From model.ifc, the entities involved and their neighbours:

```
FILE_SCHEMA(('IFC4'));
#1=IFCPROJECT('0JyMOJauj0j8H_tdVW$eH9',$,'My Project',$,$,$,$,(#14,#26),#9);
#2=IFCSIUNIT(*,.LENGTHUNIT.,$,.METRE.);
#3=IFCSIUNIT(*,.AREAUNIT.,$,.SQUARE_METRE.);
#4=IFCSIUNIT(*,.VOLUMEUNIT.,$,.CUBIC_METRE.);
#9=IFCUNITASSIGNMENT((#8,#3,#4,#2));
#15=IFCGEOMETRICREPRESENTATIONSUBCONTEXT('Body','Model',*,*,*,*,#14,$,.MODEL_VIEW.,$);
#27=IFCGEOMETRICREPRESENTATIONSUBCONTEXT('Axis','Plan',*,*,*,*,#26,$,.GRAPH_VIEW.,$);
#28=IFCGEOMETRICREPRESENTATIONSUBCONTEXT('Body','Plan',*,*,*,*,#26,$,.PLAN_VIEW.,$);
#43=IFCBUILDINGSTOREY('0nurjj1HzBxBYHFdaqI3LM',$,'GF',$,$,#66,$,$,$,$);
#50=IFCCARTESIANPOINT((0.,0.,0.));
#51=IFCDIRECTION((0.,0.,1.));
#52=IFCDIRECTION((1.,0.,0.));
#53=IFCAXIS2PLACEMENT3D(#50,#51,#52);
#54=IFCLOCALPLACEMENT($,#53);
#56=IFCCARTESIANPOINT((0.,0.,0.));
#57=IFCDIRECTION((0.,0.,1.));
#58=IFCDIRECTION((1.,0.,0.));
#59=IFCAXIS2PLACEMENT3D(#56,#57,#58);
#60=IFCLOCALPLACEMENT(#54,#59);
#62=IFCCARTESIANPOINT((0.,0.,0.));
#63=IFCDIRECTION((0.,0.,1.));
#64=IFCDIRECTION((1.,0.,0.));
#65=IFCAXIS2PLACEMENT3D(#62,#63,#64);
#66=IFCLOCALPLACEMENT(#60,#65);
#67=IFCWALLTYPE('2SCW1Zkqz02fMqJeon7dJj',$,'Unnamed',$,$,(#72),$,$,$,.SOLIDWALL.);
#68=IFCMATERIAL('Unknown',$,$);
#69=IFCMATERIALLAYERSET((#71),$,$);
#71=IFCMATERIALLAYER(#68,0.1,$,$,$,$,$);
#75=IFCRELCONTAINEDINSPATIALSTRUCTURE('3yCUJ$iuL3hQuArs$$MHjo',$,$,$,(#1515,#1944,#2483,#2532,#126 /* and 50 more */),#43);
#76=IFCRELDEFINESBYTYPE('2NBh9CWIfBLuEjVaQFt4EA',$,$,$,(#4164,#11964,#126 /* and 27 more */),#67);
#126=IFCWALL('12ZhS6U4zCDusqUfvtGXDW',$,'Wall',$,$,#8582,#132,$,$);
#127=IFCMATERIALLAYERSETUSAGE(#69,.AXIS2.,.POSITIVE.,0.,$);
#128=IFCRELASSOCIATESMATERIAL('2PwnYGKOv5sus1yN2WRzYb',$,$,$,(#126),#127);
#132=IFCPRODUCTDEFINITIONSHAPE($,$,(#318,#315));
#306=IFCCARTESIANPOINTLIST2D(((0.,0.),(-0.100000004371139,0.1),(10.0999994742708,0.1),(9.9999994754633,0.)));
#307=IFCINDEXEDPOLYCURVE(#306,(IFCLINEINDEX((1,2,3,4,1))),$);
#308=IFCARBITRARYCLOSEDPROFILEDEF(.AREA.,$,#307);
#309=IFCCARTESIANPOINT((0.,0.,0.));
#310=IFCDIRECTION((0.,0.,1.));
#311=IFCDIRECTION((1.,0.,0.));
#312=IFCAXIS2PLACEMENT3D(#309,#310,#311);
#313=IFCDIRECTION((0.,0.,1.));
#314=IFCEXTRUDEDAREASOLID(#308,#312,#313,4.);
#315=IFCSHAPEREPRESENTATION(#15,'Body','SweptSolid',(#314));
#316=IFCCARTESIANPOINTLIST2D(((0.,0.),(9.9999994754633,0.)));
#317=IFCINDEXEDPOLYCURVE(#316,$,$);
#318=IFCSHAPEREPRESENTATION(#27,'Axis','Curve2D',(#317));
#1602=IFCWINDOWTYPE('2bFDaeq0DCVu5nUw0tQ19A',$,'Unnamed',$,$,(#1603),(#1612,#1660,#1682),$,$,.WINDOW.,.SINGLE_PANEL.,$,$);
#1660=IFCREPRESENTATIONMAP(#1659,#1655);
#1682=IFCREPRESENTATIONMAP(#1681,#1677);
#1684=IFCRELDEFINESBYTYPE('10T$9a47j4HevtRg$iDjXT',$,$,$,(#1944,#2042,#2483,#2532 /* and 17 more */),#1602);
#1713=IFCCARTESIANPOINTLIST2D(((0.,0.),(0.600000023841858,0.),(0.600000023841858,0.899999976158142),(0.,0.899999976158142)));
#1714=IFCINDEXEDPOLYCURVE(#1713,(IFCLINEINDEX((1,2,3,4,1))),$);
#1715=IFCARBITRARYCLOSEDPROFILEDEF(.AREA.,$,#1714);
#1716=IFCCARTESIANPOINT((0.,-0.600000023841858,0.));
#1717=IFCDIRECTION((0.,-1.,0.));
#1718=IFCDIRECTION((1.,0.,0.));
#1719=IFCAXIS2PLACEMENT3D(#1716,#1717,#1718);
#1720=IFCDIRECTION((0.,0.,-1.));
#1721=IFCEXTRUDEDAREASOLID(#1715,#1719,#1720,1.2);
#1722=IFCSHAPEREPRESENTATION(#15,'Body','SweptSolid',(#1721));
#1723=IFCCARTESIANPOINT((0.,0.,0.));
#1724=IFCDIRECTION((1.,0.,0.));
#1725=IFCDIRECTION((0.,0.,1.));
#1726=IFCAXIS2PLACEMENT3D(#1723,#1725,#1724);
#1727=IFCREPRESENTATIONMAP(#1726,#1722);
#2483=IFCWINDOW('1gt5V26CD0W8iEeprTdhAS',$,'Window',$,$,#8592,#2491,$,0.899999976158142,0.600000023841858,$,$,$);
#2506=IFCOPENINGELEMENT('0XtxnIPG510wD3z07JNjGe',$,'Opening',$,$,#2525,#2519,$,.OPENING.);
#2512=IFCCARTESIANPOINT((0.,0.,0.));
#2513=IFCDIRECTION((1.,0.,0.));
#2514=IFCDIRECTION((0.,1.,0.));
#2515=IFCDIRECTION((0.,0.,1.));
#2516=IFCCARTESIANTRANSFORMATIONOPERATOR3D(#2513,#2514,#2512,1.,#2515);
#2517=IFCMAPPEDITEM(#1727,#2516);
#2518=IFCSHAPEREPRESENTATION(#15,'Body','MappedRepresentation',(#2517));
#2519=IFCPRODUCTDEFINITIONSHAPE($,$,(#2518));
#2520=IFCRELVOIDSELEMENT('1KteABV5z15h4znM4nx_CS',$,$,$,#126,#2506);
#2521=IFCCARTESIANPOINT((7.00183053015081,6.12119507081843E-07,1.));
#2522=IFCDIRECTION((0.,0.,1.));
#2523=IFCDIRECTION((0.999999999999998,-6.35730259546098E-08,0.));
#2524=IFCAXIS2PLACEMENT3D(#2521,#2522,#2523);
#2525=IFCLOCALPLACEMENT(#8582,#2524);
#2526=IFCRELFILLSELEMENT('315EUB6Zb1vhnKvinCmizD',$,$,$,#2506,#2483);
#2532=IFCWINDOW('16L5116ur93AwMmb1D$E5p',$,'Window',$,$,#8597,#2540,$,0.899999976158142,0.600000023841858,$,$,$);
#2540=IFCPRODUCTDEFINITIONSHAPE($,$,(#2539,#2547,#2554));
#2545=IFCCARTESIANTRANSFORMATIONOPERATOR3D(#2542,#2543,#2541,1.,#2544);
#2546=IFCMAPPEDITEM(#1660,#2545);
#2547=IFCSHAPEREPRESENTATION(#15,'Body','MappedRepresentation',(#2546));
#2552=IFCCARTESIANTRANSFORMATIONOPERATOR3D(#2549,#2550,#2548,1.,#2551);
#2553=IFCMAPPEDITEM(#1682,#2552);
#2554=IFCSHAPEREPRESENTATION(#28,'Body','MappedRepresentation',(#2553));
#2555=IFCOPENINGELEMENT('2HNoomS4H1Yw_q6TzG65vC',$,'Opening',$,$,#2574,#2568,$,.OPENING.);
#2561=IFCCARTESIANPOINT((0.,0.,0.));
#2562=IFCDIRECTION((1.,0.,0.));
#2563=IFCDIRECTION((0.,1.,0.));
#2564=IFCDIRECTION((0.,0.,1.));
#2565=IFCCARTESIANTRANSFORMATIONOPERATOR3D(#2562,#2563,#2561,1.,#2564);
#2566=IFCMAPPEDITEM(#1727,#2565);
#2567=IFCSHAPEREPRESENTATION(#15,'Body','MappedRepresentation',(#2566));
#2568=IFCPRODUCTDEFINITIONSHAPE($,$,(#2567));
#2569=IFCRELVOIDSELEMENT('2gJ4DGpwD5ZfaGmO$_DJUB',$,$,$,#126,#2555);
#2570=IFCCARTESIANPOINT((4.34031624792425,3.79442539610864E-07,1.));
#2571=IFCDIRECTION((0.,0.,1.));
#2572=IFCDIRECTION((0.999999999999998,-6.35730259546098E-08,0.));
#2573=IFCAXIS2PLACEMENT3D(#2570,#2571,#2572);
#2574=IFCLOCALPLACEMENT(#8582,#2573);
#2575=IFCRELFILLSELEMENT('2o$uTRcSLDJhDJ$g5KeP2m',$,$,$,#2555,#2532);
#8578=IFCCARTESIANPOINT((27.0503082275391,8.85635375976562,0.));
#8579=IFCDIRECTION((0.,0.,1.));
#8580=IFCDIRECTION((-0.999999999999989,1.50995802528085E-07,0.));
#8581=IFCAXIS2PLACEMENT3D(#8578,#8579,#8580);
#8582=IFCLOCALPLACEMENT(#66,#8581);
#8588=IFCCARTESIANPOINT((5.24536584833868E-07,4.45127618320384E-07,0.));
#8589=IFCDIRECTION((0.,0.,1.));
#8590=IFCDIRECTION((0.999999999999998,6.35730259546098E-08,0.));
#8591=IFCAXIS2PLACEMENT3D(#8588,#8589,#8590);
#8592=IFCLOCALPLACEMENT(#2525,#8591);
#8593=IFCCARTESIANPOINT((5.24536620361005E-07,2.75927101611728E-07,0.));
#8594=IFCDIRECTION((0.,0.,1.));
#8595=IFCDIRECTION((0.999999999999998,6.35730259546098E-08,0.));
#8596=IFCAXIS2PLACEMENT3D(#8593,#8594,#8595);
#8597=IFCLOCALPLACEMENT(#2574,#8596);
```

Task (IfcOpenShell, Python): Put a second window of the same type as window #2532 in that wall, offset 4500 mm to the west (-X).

```python
import ifcopenshell
import ifcopenshell.api.feature
import ifcopenshell.api.geometry
import ifcopenshell.api.root
import ifcopenshell.geom
import ifcopenshell.util.element
import ifcopenshell.util.placement
import ifcopenshell.util.shape
import ifcopenshell.util.unit

model = ifcopenshell.open("model.ifc")
unit_scale = ifcopenshell.util.unit.calculate_unit_scale(model)
settings = ifcopenshell.geom.settings()


def volume(element):
    """Net volume in cubic metres, openings subtracted."""
    shape = ifcopenshell.geom.create_shape(settings, element)
    return ifcopenshell.util.shape.get_volume(shape.geometry)


window = model.by_id(2532)
opening = window.FillsVoids[0].RelatingOpeningElement
wall = opening.VoidsElements[0].RelatingBuildingElement
before = volume(wall)
shift = ifcopenshell.util.placement.get_local_placement(wall.ObjectPlacement)[:3, 0] * 4.5 / unit_scale

# copy_class copies the void relationship, type, container and properties, but no geometry.
new_opening = ifcopenshell.api.root.copy_class(model, product=opening)
new_opening.Representation = ifcopenshell.util.element.copy_deep(
    model, opening.Representation, exclude=["IfcGeometricRepresentationContext", "IfcRepresentationMap"]
)
new_window = ifcopenshell.api.root.copy_class(model, product=window)
new_window.Representation = ifcopenshell.util.element.copy_deep(
    model, window.Representation, exclude=["IfcGeometricRepresentationContext", "IfcRepresentationMap"]
)
ifcopenshell.api.feature.add_filling(model, opening=new_opening, element=new_window)

for old, new in ((opening, new_opening), (window, new_window)):
    matrix = ifcopenshell.util.placement.get_local_placement(old.ObjectPlacement)
    matrix[:3, 3] += shift
    ifcopenshell.api.geometry.edit_object_placement(model, product=new, matrix=matrix, is_si=False)

after = volume(wall)

print(f"wall volume {before:.3f} -> {after:.3f} m3")

model.write("model_edited.ifc")
```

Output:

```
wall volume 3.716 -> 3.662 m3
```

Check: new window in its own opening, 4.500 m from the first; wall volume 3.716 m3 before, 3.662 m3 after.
